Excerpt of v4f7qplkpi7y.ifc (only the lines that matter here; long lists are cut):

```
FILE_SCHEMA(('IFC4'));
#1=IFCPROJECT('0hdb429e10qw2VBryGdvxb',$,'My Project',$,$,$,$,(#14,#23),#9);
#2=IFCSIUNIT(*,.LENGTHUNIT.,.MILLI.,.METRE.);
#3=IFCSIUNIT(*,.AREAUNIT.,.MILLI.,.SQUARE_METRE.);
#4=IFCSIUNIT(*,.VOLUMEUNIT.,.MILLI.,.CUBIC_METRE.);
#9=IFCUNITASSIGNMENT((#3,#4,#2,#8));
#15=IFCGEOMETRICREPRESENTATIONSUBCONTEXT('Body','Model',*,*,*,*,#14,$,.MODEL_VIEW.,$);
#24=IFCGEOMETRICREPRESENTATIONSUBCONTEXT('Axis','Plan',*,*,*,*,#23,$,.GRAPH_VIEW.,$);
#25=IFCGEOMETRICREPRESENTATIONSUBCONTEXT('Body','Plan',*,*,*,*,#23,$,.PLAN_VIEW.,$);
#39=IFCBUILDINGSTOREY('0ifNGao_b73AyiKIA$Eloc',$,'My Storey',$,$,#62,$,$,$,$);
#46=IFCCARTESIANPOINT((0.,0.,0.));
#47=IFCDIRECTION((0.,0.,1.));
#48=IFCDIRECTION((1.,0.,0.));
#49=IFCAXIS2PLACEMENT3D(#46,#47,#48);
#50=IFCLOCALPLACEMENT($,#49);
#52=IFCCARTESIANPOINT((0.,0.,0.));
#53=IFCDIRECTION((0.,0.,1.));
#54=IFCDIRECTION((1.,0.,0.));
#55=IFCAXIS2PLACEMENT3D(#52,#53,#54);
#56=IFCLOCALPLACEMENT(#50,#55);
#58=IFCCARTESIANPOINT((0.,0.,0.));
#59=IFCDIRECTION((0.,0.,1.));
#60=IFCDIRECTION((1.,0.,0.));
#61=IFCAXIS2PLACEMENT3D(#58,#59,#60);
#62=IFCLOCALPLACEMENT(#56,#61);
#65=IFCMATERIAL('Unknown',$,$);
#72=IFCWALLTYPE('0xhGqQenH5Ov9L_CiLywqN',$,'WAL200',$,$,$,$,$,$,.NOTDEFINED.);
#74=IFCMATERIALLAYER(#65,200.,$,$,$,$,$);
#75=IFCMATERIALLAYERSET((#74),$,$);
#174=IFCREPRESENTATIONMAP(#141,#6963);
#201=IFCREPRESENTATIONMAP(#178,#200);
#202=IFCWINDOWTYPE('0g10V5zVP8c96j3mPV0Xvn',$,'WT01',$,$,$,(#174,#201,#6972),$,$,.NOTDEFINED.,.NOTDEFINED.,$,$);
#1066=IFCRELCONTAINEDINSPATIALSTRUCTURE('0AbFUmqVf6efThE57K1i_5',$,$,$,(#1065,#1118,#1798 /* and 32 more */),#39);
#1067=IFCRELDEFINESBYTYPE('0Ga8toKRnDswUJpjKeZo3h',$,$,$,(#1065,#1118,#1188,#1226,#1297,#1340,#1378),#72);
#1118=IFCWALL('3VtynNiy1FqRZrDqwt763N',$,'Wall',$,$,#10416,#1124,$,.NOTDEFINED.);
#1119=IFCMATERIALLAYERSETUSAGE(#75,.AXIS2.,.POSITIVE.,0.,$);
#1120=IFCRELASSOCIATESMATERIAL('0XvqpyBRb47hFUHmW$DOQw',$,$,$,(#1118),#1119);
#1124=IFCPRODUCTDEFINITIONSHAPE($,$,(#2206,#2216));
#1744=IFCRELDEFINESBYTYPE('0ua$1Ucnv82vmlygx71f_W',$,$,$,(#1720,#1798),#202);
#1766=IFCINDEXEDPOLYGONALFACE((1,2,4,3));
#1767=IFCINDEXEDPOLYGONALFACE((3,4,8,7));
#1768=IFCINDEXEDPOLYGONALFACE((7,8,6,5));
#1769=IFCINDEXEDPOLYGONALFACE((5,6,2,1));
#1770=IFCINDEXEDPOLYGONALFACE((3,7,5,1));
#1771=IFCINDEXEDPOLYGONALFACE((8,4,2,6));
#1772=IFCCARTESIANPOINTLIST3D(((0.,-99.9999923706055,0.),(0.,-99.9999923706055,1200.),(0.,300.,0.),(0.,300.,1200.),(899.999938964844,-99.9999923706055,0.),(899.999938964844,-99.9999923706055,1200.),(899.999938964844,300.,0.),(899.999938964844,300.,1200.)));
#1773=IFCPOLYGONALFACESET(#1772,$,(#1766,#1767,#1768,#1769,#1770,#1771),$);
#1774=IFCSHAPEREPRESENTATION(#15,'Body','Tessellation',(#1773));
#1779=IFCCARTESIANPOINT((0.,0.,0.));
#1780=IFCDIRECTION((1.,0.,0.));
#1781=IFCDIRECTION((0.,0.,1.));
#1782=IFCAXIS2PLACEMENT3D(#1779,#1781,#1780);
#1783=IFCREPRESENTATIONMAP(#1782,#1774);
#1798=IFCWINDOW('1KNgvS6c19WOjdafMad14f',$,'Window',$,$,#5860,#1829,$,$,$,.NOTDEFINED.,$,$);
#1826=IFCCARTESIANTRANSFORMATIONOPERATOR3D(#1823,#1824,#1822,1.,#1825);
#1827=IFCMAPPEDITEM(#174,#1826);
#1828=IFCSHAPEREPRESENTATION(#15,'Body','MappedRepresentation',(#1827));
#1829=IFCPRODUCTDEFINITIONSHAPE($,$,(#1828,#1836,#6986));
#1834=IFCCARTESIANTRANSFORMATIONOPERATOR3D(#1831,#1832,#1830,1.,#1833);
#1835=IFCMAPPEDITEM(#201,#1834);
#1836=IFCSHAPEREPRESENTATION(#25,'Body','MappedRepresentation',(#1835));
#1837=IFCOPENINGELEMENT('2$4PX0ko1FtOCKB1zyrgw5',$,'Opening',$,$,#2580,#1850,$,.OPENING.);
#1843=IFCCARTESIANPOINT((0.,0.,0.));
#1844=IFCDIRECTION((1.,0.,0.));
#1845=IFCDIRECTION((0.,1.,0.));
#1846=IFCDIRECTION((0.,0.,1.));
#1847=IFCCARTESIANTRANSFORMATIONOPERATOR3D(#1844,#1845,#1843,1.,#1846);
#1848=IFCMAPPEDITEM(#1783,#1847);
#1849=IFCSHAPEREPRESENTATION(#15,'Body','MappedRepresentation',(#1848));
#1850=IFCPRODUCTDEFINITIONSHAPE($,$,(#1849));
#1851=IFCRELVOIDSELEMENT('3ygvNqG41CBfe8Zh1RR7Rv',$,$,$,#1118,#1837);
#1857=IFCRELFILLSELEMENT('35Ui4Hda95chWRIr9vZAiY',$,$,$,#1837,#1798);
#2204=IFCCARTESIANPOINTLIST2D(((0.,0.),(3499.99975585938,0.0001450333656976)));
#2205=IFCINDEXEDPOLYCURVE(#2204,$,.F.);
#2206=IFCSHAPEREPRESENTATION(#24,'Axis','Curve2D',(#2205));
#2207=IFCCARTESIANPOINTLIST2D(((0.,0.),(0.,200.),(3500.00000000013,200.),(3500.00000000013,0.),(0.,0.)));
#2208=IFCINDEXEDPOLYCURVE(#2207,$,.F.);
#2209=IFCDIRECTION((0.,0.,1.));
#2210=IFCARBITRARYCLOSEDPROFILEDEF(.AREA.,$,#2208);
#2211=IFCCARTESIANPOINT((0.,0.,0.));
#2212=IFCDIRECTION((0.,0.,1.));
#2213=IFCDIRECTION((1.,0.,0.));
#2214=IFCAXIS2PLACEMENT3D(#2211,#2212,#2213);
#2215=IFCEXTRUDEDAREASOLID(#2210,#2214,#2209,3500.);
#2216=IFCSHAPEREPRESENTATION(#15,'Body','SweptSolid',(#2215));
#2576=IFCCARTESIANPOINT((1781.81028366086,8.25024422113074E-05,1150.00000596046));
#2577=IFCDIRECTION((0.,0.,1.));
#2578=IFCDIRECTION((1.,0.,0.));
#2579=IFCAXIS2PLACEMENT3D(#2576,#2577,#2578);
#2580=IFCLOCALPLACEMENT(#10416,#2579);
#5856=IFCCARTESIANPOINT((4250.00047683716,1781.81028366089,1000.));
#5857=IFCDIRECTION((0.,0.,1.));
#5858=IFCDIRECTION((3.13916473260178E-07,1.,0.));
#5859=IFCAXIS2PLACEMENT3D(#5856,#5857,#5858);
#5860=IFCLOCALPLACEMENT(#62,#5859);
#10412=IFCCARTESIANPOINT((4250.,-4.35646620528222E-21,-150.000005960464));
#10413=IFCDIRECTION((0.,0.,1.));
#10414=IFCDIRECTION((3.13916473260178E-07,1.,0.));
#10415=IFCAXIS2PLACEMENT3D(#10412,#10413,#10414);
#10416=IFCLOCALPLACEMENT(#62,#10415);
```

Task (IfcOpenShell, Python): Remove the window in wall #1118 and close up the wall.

```python
import ifcopenshell
import ifcopenshell.api.feature
import ifcopenshell.api.root
import ifcopenshell.geom
import ifcopenshell.util.shape

model = ifcopenshell.open("v4f7qplkpi7y.ifc")
settings = ifcopenshell.geom.settings()


def volume(element):
    """Net volume in cubic metres, openings subtracted."""
    shape = ifcopenshell.geom.create_shape(settings, element)
    return ifcopenshell.util.shape.get_volume(shape.geometry)


window = model.by_id(1798)
opening = window.FillsVoids[0].RelatingOpeningElement
wall = opening.VoidsElements[0].RelatingBuildingElement
before = volume(wall)

ifcopenshell.api.root.remove_product(model, product=window)
ifcopenshell.api.feature.remove_feature(model, feature=opening)

after = volume(wall)

print(f"wall volume {before:.3f} -> {after:.3f} m3")

model.write("v4f7qplkpi7y_rev.ifc")
```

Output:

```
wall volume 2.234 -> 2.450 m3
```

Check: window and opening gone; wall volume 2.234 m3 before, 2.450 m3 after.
